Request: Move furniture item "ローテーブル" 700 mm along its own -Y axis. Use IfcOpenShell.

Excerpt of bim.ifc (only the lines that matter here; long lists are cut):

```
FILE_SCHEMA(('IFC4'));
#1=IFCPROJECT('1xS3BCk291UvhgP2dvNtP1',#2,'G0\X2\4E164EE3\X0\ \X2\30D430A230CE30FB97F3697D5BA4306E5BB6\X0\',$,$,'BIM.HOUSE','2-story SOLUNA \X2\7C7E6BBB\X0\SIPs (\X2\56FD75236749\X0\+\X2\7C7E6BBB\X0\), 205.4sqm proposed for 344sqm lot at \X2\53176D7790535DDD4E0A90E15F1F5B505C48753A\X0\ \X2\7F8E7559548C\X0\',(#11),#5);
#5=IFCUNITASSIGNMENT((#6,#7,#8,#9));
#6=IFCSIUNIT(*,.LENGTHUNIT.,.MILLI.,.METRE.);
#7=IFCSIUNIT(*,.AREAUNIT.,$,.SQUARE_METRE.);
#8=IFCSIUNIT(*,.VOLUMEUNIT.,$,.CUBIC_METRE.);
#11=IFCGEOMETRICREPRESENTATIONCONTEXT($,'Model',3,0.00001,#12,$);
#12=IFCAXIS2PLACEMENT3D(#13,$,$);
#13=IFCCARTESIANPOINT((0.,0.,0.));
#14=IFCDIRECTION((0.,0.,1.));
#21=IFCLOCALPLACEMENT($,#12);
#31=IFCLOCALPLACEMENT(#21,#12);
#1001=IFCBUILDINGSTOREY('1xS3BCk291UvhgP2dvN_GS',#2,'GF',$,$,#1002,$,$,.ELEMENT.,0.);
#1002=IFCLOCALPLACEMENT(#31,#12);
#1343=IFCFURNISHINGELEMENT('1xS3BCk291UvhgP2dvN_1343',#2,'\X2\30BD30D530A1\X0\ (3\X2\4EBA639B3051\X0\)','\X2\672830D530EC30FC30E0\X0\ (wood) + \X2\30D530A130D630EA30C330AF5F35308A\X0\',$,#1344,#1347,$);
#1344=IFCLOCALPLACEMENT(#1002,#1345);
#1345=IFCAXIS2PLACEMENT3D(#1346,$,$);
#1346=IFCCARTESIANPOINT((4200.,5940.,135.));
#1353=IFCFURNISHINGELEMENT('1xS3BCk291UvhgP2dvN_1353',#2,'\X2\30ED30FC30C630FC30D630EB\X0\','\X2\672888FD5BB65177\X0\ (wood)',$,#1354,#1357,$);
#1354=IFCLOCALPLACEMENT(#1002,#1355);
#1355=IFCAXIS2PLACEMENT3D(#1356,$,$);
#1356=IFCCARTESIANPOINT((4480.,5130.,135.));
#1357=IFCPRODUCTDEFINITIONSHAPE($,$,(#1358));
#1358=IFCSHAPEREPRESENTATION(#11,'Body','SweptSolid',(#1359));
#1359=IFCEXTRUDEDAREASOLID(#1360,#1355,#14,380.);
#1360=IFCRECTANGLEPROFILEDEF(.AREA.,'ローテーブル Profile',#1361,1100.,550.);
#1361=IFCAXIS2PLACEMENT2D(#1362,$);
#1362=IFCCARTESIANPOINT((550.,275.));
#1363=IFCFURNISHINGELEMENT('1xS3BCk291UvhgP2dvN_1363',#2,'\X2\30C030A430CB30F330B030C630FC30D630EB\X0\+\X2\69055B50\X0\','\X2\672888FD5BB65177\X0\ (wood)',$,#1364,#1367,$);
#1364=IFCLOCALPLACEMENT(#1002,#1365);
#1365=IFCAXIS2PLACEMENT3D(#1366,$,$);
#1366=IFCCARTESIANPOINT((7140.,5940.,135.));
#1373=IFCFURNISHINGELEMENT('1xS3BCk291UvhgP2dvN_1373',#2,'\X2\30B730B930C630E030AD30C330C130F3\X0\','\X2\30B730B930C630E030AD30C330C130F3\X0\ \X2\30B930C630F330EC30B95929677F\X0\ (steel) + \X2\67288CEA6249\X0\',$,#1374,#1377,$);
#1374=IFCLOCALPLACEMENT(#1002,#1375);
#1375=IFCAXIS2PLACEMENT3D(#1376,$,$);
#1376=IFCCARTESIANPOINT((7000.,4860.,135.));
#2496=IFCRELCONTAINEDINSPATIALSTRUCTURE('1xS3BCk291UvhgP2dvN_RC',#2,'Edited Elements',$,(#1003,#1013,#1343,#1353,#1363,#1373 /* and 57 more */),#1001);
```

```python
import ifcopenshell
import ifcopenshell.api.geometry
import ifcopenshell.util.placement
import ifcopenshell.util.unit

model = ifcopenshell.open("bim.ifc")
unit_scale = ifcopenshell.util.unit.calculate_unit_scale(model)

item = model.by_id(1353)
matrix = ifcopenshell.util.placement.get_local_placement(item.ObjectPlacement)
matrix[:3, 3] -= matrix[:3, 1] * 0.7 / unit_scale
ifcopenshell.api.geometry.edit_object_placement(model, product=item, matrix=matrix, is_si=False)

print(ifcopenshell.util.placement.get_local_placement(item.ObjectPlacement).round(3) + 0.0)

model.write("bim_v2.ifc")
```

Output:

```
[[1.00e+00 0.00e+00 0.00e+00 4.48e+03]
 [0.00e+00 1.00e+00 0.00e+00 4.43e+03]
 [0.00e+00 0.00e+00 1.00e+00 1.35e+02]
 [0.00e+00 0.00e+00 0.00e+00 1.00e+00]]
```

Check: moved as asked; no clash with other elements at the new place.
